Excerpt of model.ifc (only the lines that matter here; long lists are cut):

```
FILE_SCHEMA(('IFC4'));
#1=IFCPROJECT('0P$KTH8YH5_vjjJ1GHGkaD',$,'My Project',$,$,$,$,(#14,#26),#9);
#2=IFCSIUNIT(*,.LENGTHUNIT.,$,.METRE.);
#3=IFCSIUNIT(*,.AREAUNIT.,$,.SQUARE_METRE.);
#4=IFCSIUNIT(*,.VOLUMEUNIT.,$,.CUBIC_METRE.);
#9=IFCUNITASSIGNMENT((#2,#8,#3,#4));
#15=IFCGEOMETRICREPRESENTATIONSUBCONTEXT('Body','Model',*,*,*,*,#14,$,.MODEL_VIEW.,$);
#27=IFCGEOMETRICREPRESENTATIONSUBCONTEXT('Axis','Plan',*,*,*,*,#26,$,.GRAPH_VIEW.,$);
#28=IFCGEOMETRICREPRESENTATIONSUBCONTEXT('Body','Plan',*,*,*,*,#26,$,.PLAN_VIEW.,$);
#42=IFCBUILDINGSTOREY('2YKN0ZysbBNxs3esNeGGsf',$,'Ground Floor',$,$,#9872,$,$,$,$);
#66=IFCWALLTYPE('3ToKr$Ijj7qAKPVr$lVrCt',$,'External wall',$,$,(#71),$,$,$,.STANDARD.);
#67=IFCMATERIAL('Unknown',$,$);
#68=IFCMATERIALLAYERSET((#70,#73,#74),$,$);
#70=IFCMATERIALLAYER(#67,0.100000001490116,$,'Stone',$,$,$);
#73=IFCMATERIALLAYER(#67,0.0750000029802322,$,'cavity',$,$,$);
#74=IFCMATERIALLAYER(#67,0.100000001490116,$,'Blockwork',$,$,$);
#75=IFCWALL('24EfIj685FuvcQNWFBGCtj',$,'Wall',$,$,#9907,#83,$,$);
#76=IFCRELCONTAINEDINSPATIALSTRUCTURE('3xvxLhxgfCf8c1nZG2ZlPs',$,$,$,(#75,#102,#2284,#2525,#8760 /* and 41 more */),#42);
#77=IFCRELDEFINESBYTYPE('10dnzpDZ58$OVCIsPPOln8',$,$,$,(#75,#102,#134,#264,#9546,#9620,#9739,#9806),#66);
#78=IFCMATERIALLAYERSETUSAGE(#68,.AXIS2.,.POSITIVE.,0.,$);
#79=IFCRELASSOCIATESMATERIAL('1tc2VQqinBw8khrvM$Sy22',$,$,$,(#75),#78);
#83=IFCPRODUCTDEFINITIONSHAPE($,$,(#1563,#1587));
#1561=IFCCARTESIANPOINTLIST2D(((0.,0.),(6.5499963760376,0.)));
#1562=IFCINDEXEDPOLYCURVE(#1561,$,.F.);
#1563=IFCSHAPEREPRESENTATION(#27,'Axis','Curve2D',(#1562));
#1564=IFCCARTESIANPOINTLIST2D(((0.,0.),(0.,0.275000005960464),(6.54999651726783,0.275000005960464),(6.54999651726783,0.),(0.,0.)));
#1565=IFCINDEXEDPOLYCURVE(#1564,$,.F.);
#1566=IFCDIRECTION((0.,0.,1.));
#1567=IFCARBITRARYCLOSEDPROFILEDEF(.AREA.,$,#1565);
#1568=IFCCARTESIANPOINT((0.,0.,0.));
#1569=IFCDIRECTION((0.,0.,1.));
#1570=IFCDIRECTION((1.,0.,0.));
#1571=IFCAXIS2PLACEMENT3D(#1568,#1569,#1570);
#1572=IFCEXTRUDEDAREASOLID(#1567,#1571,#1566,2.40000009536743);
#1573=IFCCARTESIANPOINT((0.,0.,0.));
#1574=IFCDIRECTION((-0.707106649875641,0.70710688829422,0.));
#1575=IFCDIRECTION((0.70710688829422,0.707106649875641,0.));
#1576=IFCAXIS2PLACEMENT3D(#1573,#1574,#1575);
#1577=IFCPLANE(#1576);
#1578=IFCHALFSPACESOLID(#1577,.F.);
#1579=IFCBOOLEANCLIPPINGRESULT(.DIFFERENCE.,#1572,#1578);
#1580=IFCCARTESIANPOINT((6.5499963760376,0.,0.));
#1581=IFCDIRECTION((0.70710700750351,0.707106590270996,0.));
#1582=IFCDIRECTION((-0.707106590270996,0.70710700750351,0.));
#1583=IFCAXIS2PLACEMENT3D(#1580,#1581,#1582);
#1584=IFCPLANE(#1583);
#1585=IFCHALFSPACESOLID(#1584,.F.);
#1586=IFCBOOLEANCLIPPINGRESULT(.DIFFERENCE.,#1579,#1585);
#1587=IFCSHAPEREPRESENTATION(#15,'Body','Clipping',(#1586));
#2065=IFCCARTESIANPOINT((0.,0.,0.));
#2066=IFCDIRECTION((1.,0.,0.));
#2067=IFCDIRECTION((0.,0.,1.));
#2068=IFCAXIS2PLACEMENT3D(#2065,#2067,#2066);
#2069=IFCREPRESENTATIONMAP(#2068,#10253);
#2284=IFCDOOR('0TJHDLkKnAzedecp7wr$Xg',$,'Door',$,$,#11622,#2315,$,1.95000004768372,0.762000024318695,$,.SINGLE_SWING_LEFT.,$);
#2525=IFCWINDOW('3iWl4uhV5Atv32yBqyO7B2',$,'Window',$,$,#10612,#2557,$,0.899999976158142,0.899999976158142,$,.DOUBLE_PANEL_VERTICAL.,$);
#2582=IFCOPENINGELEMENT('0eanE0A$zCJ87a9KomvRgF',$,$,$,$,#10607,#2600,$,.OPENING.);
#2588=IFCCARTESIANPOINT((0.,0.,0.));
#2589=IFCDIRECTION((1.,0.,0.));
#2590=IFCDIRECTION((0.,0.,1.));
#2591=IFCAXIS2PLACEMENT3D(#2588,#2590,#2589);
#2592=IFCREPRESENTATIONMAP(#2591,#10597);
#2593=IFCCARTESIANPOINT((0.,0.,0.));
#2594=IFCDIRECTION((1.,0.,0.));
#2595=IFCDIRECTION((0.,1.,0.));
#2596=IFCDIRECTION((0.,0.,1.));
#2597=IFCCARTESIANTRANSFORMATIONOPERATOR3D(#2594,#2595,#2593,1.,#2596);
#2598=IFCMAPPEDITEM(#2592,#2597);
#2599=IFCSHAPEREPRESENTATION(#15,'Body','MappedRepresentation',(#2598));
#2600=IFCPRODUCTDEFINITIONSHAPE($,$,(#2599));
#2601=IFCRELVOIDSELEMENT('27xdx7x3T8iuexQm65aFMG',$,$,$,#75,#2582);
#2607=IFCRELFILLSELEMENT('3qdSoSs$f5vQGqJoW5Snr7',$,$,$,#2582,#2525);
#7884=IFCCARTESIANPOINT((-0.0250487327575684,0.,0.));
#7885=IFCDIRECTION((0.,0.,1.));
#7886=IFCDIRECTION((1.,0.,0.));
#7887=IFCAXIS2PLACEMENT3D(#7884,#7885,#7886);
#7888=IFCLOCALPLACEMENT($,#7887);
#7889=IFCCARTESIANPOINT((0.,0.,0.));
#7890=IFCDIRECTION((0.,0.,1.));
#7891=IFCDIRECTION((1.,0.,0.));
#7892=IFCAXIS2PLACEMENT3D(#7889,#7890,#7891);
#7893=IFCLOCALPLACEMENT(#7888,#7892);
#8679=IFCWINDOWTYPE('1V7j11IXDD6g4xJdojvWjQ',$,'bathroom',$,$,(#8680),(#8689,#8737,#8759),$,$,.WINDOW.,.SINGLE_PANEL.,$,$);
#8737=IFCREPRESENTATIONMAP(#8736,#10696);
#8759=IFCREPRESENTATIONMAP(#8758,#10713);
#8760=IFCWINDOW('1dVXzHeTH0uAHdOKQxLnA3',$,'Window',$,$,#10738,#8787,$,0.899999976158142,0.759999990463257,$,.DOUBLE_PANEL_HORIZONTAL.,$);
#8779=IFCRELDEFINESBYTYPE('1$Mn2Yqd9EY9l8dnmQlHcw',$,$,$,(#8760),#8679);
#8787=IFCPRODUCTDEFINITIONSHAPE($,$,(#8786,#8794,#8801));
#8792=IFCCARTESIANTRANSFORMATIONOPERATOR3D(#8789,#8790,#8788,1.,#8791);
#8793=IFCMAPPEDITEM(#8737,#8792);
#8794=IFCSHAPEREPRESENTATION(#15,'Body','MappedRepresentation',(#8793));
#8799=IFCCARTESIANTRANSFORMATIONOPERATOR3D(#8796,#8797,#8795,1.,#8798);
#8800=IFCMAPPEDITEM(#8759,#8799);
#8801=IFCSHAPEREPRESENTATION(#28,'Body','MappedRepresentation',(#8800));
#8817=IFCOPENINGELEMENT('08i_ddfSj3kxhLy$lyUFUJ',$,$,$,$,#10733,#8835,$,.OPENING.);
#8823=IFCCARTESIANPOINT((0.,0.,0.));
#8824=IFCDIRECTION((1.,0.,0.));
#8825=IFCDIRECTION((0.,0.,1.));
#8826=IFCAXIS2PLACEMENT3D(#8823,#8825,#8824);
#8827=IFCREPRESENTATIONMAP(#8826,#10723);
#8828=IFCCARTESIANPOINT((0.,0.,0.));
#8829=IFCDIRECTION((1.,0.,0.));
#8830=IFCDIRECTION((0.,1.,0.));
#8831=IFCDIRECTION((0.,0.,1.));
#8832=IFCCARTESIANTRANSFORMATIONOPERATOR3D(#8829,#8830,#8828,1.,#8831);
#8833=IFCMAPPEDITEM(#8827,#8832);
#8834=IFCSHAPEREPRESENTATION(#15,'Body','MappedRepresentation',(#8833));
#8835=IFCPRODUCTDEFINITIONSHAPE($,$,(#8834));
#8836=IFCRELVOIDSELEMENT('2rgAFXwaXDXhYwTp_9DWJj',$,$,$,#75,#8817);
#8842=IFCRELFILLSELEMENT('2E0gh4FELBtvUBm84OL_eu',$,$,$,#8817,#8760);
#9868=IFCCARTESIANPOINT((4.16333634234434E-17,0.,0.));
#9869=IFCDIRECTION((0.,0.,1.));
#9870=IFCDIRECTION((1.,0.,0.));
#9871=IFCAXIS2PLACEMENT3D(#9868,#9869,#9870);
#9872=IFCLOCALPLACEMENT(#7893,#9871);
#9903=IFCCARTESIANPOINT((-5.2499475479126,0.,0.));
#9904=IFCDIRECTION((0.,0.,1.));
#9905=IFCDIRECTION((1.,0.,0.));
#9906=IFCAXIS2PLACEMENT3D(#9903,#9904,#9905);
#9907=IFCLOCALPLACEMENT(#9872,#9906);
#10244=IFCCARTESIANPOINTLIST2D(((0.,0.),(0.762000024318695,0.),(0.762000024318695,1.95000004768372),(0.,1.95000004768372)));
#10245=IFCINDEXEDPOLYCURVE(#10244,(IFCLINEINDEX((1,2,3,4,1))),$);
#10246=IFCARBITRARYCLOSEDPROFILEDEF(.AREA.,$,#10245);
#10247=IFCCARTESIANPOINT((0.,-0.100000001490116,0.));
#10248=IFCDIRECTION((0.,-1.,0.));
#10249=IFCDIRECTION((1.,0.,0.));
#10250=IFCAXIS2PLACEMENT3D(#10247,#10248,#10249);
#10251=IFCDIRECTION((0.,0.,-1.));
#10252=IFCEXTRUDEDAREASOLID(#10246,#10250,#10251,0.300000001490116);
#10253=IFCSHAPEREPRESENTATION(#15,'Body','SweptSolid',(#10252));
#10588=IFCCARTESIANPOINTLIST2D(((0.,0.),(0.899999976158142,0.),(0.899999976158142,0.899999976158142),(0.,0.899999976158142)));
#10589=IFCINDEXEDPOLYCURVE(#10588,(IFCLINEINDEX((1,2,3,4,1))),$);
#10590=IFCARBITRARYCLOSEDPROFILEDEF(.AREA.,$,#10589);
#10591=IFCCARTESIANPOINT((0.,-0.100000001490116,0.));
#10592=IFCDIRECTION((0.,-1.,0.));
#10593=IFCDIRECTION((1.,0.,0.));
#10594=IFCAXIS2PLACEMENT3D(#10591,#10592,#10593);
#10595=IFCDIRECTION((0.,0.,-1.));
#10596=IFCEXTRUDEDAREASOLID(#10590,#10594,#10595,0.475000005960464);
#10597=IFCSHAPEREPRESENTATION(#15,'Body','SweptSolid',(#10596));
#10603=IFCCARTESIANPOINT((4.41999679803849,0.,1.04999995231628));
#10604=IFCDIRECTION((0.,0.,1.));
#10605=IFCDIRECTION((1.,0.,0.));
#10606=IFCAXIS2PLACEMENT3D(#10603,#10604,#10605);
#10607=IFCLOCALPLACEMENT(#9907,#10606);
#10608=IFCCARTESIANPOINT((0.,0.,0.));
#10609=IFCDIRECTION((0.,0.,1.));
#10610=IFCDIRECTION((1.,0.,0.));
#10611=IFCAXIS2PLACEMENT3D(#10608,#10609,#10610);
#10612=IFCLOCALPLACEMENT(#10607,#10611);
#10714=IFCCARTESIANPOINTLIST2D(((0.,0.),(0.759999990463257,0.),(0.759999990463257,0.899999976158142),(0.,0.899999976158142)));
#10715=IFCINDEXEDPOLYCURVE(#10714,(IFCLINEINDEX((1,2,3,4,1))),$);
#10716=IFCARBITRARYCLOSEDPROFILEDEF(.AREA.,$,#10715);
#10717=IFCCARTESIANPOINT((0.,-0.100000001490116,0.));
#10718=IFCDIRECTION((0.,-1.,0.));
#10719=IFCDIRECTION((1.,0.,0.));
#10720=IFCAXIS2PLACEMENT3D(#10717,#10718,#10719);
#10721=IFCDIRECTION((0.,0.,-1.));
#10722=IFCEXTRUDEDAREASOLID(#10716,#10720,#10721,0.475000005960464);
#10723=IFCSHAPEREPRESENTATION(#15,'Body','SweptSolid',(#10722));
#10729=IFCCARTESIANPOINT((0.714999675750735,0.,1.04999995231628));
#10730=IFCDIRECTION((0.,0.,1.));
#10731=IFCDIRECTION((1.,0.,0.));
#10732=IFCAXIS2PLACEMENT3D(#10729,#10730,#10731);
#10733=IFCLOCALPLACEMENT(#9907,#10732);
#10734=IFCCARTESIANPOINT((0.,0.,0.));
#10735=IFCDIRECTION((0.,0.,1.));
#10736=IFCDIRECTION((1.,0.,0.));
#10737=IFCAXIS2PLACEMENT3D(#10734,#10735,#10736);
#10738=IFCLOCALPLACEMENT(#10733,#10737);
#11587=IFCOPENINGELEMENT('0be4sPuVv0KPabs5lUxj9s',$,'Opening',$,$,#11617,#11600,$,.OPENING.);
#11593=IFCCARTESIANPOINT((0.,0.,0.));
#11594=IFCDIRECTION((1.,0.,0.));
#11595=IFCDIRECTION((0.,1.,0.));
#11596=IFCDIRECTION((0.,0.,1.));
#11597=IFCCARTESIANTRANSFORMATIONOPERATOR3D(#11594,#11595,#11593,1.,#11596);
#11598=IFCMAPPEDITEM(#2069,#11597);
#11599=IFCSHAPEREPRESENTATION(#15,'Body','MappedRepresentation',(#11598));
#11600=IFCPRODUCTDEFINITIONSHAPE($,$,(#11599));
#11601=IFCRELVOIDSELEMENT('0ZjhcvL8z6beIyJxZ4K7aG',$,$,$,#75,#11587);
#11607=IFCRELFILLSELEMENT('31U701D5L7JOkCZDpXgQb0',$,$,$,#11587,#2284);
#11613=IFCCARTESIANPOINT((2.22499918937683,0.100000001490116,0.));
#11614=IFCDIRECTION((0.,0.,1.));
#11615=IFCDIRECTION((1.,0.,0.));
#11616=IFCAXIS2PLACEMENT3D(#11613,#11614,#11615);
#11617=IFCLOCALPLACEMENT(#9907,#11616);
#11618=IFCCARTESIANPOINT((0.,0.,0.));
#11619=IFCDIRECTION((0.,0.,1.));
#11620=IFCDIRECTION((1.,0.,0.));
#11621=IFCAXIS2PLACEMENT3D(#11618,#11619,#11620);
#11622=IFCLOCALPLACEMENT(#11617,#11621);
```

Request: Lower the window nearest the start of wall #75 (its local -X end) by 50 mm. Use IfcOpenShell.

```python
import numpy as np
import ifcopenshell
import ifcopenshell.api.geometry
import ifcopenshell.util.placement
import ifcopenshell.util.unit

model = ifcopenshell.open("model.ifc")
unit_scale = ifcopenshell.util.unit.calculate_unit_scale(model)

window = model.by_guid("1dVXzHeTH0uAHdOKQxLnA3")
opening = window.FillsVoids[0].RelatingOpeningElement
dz = -0.05 / unit_scale

shift = np.array([0.0, 0.0, dz])
# The window is placed relative to its opening, so it follows when the opening moves.
matrix = ifcopenshell.util.placement.get_local_placement(opening.ObjectPlacement)
matrix[:3, 3] += shift
ifcopenshell.api.geometry.edit_object_placement(
    model, product=opening, matrix=matrix, is_si=False, should_transform_children=True
)

print(f"moved by {dz * unit_scale:+.3f} m")

model.write("model_v2.ifc")
```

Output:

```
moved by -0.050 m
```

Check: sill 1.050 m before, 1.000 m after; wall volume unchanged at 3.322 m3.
